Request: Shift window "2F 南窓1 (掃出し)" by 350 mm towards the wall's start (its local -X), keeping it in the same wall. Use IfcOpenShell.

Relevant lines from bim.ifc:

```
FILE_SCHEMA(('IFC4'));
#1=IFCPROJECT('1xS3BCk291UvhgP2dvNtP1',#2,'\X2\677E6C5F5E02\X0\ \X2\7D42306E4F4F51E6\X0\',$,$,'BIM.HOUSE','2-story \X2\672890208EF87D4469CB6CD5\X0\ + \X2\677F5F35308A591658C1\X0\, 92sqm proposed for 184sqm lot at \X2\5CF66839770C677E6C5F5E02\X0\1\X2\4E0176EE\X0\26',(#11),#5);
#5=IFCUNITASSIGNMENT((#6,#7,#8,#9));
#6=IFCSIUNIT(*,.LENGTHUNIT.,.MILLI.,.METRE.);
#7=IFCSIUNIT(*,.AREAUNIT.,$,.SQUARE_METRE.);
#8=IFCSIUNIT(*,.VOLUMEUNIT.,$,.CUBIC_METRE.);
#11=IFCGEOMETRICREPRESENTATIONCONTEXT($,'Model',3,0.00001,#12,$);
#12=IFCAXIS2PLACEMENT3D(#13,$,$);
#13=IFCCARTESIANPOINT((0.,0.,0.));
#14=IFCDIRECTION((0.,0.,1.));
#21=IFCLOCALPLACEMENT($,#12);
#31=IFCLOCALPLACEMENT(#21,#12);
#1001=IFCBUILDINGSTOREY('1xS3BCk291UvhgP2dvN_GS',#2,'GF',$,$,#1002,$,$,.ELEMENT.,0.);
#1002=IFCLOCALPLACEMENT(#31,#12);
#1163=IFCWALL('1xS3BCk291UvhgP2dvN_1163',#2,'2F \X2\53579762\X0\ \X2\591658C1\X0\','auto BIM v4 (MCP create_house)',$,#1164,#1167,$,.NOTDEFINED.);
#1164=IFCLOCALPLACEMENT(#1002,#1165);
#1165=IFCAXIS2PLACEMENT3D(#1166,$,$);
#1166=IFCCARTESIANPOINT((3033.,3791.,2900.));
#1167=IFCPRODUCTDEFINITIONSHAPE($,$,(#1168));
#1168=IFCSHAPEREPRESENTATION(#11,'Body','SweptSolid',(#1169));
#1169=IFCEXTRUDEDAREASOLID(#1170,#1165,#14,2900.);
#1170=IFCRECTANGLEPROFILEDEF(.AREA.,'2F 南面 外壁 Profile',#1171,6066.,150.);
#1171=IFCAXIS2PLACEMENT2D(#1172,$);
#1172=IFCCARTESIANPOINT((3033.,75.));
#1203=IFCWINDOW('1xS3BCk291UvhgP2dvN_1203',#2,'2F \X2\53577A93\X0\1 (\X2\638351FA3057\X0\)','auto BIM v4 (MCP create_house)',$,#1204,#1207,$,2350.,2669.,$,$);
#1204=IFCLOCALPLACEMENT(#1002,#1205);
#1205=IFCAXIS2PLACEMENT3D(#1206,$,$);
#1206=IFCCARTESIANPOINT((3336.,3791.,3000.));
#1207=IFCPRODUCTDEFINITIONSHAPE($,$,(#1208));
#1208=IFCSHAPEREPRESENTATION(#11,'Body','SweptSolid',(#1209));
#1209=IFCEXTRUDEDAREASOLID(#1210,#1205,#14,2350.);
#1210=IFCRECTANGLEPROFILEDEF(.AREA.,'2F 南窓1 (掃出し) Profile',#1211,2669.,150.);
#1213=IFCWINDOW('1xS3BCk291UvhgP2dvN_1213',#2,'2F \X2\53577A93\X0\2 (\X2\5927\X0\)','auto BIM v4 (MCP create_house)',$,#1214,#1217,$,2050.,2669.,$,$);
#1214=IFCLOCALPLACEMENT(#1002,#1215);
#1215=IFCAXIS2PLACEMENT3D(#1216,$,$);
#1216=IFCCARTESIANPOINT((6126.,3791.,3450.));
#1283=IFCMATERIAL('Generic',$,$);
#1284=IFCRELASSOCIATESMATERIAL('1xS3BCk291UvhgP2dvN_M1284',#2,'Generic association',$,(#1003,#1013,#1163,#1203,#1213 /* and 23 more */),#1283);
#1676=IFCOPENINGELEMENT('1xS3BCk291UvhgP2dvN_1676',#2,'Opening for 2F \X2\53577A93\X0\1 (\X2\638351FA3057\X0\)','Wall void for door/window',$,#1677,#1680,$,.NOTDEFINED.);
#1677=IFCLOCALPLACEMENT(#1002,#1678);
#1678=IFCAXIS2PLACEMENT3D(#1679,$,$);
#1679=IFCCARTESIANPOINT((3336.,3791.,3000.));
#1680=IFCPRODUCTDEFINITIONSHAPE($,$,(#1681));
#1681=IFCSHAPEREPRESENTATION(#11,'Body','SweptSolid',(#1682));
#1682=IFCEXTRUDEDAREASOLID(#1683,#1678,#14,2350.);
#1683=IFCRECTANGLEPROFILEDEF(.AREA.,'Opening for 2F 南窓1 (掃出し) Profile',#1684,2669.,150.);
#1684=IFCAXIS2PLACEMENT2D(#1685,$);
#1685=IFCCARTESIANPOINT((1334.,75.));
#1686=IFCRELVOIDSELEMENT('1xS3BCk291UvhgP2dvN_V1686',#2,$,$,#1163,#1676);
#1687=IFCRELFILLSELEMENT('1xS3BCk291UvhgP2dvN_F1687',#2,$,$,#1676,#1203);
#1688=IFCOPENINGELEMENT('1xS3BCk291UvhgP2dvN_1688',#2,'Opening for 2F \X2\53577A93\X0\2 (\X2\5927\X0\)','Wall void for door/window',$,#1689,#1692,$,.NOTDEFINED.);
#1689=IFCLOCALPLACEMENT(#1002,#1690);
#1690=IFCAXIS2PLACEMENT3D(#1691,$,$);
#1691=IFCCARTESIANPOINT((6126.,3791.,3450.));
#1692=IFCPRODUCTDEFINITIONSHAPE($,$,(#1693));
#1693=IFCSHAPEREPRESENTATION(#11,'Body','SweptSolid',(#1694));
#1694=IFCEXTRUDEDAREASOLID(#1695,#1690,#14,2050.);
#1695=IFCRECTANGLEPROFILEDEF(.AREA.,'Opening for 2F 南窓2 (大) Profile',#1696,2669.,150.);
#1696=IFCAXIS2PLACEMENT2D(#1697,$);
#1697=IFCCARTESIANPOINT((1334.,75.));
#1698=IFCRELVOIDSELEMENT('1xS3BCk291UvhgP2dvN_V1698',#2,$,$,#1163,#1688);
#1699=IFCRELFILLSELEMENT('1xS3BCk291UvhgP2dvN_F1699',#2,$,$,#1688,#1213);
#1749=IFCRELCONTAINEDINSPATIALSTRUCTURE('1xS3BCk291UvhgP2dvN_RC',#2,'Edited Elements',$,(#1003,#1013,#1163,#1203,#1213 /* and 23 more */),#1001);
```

```python
import ifcopenshell
import ifcopenshell.api.geometry
import ifcopenshell.util.placement

model = ifcopenshell.open("bim.ifc")

window = model.by_guid("1xS3BCk291UvhgP2dvN_1203")
opening = window.FillsVoids[0].RelatingOpeningElement
wall = opening.VoidsElements[0].RelatingBuildingElement

wall_matrix = ifcopenshell.util.placement.get_local_placement(wall.ObjectPlacement)
shift = wall_matrix[:3, 0] * -350.0
before = ifcopenshell.util.placement.get_local_placement(window.ObjectPlacement)[:3, 3].copy()

# The window is not placed relative to its opening, so move both.
for product in (opening, window):
    matrix = ifcopenshell.util.placement.get_local_placement(product.ObjectPlacement)
    matrix[:3, 3] += shift
    ifcopenshell.api.geometry.edit_object_placement(model, product=product, matrix=matrix, is_si=False)

after = ifcopenshell.util.placement.get_local_placement(window.ObjectPlacement)[:3, 3]
print("window moved by", (after - before).round(3) + 0.0)

model.write("bim_edited.ifc")
```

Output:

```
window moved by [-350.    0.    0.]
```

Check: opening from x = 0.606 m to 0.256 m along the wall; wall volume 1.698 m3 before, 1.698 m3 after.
